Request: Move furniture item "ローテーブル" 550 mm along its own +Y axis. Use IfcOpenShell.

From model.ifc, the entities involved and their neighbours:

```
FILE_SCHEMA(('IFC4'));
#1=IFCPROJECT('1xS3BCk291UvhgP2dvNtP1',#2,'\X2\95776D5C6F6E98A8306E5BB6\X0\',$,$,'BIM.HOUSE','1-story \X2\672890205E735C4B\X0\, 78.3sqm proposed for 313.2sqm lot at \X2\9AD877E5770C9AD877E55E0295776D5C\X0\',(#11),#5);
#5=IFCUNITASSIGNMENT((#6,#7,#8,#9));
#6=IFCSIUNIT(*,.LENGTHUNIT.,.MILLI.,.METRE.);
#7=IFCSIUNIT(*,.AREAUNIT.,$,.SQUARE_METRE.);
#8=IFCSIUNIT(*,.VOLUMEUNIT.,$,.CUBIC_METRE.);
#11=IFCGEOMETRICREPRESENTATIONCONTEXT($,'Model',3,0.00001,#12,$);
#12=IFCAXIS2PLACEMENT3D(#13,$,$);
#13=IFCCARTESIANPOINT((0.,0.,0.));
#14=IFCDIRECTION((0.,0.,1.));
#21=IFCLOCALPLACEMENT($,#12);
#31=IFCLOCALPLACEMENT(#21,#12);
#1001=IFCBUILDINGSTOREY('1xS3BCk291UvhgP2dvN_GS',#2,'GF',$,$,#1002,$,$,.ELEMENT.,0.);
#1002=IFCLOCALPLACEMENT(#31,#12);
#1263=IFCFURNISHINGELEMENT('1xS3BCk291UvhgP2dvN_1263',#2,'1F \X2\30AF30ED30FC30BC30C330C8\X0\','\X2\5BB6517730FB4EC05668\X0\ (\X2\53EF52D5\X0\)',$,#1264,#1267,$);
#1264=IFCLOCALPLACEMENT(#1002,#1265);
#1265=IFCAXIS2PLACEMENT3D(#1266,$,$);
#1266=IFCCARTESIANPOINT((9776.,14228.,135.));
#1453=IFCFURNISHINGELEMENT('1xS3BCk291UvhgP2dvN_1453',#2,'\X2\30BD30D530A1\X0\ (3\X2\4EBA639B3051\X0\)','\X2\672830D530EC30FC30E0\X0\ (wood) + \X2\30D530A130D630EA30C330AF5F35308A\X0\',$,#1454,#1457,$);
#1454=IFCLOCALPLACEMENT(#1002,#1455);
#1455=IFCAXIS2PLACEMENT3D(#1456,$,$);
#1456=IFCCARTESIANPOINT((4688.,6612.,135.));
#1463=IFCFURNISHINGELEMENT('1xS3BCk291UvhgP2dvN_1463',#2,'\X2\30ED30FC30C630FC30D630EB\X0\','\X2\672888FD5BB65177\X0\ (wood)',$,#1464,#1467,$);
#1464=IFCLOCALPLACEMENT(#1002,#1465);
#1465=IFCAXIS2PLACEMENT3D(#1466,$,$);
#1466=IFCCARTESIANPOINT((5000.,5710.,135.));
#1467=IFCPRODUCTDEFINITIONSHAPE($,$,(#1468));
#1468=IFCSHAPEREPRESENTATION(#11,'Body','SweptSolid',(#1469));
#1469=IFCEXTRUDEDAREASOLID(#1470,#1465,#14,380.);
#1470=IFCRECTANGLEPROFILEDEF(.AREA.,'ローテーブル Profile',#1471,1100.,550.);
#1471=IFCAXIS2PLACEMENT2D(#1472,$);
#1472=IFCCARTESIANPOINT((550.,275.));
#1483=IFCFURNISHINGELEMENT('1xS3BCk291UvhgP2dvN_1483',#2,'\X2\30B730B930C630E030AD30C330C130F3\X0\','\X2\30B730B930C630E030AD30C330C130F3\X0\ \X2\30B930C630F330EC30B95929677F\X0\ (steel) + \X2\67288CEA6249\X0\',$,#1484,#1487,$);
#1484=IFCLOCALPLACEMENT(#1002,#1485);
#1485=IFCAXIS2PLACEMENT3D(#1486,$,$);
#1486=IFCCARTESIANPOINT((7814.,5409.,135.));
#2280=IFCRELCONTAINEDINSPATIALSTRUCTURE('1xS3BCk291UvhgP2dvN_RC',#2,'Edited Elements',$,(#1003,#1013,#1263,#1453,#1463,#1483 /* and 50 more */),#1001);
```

```python
import ifcopenshell
import ifcopenshell.api.geometry
import ifcopenshell.util.placement

model = ifcopenshell.open("model.ifc")

item = model.by_guid("1xS3BCk291UvhgP2dvN_1463")
matrix = ifcopenshell.util.placement.get_local_placement(item.ObjectPlacement)
matrix[:3, 3] += matrix[:3, 1] * 550.0
ifcopenshell.api.geometry.edit_object_placement(model, product=item, matrix=matrix, is_si=False)

print(ifcopenshell.util.placement.get_local_placement(item.ObjectPlacement).round(3) + 0.0)

model.write("model-out.ifc")
```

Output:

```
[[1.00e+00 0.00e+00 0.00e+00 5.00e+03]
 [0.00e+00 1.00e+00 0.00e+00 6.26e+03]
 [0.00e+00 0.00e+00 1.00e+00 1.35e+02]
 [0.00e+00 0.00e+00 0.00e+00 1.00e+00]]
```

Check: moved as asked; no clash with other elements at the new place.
